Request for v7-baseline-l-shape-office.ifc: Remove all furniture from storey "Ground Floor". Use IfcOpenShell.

First a look at what the model holds.

```python
import ifcopenshell
import ifcopenshell.util.element

model = ifcopenshell.open("v7-baseline-l-shape-office.ifc")
print(model.schema)
storey = next(s for s in model.by_type("IfcBuildingStorey") if s.Name == "Ground Floor")
furniture = [e for e in ifcopenshell.util.element.get_decomposition(storey) if e.is_a("IfcFurnishingElement")]
seen = {}
for e in furniture:
    element_type = ifcopenshell.util.element.get_type(e)
    name = element_type.Name if element_type not in (None, e) else None
    seen[name] = seen.get(name, 0) + 1
for name, count in sorted(seen.items(), key=str):
    print(count, "x", name)
```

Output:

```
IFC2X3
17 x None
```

```python
import ifcopenshell
import ifcopenshell.api.root
import ifcopenshell.util.element

model = ifcopenshell.open("v7-baseline-l-shape-office.ifc")

storey = next(s for s in model.by_type("IfcBuildingStorey") if s.Name == "Ground Floor")
furniture = [e for e in ifcopenshell.util.element.get_decomposition(storey) if e.is_a("IfcFurnishingElement")]

for e in furniture:
    ifcopenshell.api.root.remove_product(model, product=e)
print(len(furniture), "removed")

model.write("v7-baseline-l-shape-office_v2.ifc")
```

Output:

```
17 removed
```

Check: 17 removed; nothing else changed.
